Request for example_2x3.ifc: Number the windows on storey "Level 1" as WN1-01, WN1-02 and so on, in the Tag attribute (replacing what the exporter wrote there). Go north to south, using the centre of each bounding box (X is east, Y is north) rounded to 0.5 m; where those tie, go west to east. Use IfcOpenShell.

First a look at what the model holds.

```python
import ifcopenshell
import ifcopenshell.util.element
import ifcopenshell.util.placement

model = ifcopenshell.open("example_2x3.ifc")
print(model.schema)
storey = next(s for s in model.by_type("IfcBuildingStorey") if s.Name == "Level 1")
windows = [e for e in ifcopenshell.util.element.get_decomposition(storey) if e.is_a("IfcWindow")]
for e in sorted(windows, key=lambda e: e.id()):
    origin = ifcopenshell.util.placement.get_local_placement(e.ObjectPlacement)[:3, 3]
    print(e.id(), e.Tag, e.Name, origin.round(2) + 0.0, sep=" | ")
```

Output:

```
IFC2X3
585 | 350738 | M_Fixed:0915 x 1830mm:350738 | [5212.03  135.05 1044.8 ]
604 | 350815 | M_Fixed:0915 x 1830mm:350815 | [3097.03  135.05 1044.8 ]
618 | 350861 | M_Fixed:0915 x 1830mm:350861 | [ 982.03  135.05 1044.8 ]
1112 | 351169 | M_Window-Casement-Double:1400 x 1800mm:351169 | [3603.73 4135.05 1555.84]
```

```python
import ifcopenshell
import ifcopenshell.geom
import ifcopenshell.util.element
import ifcopenshell.util.shape

model = ifcopenshell.open("example_2x3.ifc")
settings = ifcopenshell.geom.settings()
settings.set("use-world-coords", True)


def centre(element):
    shape = ifcopenshell.geom.create_shape(settings, element)
    return ifcopenshell.util.shape.get_bbox_centroid(shape.geometry)


storey = next(s for s in model.by_type("IfcBuildingStorey") if s.Name == "Level 1")
windows = [e for e in ifcopenshell.util.element.get_decomposition(storey) if e.is_a("IfcWindow")]

# Insertion points can sit at a corner or the storey origin, so sort by the geometry (in metres).
centres = {e: centre(e) for e in windows}
windows.sort(key=lambda e: (-round(centres[e][1] / 0.5), centres[e][0]))

for i, e in enumerate(windows, start=1):
    number = f"WN1-{i:02d}"
    e.Tag = number
    print(e.id(), number)

model.write("example_2x3-out.ifc")
```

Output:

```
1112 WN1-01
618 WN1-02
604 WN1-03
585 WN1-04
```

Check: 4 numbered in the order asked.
